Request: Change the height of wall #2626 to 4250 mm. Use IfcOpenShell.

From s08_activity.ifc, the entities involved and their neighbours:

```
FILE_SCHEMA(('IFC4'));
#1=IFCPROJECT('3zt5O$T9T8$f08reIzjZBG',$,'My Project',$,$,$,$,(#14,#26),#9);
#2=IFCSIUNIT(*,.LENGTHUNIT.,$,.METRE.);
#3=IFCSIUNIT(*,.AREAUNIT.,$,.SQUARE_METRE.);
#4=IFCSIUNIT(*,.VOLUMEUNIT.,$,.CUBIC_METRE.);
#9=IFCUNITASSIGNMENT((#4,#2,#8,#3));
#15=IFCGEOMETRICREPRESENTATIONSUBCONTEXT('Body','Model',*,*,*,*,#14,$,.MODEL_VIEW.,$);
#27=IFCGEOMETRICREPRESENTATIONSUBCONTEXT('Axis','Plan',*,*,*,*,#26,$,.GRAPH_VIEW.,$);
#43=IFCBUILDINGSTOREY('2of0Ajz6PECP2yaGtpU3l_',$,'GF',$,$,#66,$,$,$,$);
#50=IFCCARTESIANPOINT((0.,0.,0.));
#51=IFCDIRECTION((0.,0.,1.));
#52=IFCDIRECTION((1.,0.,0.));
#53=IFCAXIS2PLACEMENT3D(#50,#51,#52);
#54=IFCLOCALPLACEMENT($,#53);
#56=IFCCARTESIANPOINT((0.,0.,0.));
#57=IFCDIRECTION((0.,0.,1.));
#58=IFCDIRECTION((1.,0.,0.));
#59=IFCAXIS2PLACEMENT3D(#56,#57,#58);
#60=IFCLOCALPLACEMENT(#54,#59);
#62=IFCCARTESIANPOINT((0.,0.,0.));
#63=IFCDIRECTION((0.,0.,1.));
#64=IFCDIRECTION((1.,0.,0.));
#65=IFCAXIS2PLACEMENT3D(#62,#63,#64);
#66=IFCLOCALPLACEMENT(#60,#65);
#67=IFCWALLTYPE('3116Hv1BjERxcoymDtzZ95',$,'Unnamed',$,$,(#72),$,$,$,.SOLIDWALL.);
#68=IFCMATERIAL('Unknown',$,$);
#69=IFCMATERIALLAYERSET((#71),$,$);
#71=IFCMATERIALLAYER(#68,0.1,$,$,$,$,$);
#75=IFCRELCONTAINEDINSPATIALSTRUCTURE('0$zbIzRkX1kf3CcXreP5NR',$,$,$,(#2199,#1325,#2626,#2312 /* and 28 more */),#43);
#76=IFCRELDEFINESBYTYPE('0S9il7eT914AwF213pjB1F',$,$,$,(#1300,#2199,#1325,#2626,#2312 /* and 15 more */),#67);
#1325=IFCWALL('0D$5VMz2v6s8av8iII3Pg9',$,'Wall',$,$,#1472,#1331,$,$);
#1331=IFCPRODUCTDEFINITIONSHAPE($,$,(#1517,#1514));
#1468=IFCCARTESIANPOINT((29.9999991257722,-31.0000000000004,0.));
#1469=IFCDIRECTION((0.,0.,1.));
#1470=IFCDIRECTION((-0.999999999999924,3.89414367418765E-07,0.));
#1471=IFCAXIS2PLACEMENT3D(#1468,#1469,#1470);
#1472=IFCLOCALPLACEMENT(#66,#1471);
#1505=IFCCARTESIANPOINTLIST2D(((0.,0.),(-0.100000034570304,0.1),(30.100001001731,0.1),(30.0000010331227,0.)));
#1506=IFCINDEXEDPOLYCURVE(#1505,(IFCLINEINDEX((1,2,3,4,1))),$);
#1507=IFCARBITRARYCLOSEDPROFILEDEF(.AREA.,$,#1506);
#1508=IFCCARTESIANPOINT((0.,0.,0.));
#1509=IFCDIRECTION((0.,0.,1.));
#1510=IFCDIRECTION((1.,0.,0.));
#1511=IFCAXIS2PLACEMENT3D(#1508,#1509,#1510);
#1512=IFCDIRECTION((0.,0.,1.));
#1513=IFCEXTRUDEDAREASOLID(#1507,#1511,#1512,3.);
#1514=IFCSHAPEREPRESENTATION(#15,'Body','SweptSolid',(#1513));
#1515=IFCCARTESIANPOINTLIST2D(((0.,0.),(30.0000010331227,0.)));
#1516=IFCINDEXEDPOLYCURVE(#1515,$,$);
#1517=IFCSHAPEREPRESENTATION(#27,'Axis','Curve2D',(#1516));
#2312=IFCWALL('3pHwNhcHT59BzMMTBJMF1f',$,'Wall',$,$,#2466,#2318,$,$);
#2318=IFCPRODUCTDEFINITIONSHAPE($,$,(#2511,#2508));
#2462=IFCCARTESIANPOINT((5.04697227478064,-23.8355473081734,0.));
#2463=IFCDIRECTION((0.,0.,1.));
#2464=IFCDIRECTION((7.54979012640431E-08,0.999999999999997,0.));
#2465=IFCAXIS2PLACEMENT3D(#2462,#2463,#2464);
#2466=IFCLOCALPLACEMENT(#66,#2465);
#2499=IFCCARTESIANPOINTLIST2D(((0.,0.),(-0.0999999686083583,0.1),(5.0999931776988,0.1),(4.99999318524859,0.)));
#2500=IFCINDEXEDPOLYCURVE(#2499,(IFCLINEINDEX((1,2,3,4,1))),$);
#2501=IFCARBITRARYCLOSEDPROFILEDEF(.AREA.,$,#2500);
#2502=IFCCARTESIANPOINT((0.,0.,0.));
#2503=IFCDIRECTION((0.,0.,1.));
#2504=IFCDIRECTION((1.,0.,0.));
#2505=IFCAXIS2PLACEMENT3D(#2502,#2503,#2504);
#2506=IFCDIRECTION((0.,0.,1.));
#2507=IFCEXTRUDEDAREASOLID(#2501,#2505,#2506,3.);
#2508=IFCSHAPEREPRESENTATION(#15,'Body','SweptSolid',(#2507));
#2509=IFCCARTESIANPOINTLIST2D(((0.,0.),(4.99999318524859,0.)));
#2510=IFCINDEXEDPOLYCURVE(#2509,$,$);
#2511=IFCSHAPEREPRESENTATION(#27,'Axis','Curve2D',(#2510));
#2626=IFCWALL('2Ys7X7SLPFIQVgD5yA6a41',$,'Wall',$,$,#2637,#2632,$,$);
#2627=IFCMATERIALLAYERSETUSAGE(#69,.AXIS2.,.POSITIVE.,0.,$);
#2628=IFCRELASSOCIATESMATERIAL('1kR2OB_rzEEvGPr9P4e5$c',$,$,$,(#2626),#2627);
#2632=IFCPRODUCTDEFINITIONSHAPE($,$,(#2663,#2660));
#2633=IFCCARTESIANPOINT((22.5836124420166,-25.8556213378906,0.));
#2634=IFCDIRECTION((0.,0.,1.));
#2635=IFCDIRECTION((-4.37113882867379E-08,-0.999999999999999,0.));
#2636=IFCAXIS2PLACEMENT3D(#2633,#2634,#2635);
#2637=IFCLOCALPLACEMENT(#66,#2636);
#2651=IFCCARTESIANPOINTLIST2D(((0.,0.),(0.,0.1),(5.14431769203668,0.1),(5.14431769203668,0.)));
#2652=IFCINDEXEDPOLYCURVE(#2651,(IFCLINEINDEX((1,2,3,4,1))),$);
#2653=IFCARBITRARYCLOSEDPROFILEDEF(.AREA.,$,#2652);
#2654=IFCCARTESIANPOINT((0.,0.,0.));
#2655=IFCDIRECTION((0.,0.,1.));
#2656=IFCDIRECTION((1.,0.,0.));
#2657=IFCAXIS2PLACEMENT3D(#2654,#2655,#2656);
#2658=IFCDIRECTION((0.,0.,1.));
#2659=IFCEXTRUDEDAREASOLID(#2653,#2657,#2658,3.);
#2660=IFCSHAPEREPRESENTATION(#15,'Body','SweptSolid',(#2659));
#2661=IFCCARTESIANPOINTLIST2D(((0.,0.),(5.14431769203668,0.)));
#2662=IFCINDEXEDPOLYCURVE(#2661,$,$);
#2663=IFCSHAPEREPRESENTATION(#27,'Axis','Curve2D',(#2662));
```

```python
import ifcopenshell
import ifcopenshell.geom
import ifcopenshell.util.representation
import ifcopenshell.util.shape
import ifcopenshell.util.unit

model = ifcopenshell.open("s08_activity.ifc")
unit_scale = ifcopenshell.util.unit.calculate_unit_scale(model)
settings = ifcopenshell.geom.settings()


def volume(element):
    """Net volume in cubic metres, openings subtracted."""
    shape = ifcopenshell.geom.create_shape(settings, element)
    return ifcopenshell.util.shape.get_volume(shape.geometry)


wall = model.by_guid("2Ys7X7SLPFIQVgD5yA6a41")
before = volume(wall)

body = ifcopenshell.util.representation.get_representation(wall, "Model", "Body")
solid = body.Items[0]
old_height = solid.Depth
solid.Depth = 4.25 / unit_scale
after = volume(wall)

print(f"height {old_height:g} -> {solid.Depth:g}, volume {before:.3f} -> {after:.3f} m3")

model.write("s08_activity_rev.ifc")
```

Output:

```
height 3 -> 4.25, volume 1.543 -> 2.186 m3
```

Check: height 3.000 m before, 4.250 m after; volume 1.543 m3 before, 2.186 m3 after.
